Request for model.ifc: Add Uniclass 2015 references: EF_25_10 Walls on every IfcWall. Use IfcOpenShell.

First a look at what the model holds.

```python
import ifcopenshell

model = ifcopenshell.open("model.ifc")
print(model.schema)
print("classifications:", [c.Name for c in model.by_type("IfcClassification")])
for ifc_class in ("IfcDoor", "IfcRoof", "IfcStair", "IfcWall", "IfcWindow"):
    print(ifc_class, len(model.by_type(ifc_class)))
```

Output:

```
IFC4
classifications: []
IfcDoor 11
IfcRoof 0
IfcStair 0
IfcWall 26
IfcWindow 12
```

```python
import ifcopenshell
import ifcopenshell.api.classification

model = ifcopenshell.open("model.ifc")

system = ifcopenshell.api.classification.add_classification(model, classification="Uniclass 2015")

codes = {
    "IfcWall": ("EF_25_10", "Walls"),
}
for ifc_class, (code, name) in codes.items():
    products = model.by_type(ifc_class)
    ifcopenshell.api.classification.add_reference(
        model, products=products, classification=system, identification=code, name=name
    )
    print(code, len(products))

model.write("model_updated.ifc")
```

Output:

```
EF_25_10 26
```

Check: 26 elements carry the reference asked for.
